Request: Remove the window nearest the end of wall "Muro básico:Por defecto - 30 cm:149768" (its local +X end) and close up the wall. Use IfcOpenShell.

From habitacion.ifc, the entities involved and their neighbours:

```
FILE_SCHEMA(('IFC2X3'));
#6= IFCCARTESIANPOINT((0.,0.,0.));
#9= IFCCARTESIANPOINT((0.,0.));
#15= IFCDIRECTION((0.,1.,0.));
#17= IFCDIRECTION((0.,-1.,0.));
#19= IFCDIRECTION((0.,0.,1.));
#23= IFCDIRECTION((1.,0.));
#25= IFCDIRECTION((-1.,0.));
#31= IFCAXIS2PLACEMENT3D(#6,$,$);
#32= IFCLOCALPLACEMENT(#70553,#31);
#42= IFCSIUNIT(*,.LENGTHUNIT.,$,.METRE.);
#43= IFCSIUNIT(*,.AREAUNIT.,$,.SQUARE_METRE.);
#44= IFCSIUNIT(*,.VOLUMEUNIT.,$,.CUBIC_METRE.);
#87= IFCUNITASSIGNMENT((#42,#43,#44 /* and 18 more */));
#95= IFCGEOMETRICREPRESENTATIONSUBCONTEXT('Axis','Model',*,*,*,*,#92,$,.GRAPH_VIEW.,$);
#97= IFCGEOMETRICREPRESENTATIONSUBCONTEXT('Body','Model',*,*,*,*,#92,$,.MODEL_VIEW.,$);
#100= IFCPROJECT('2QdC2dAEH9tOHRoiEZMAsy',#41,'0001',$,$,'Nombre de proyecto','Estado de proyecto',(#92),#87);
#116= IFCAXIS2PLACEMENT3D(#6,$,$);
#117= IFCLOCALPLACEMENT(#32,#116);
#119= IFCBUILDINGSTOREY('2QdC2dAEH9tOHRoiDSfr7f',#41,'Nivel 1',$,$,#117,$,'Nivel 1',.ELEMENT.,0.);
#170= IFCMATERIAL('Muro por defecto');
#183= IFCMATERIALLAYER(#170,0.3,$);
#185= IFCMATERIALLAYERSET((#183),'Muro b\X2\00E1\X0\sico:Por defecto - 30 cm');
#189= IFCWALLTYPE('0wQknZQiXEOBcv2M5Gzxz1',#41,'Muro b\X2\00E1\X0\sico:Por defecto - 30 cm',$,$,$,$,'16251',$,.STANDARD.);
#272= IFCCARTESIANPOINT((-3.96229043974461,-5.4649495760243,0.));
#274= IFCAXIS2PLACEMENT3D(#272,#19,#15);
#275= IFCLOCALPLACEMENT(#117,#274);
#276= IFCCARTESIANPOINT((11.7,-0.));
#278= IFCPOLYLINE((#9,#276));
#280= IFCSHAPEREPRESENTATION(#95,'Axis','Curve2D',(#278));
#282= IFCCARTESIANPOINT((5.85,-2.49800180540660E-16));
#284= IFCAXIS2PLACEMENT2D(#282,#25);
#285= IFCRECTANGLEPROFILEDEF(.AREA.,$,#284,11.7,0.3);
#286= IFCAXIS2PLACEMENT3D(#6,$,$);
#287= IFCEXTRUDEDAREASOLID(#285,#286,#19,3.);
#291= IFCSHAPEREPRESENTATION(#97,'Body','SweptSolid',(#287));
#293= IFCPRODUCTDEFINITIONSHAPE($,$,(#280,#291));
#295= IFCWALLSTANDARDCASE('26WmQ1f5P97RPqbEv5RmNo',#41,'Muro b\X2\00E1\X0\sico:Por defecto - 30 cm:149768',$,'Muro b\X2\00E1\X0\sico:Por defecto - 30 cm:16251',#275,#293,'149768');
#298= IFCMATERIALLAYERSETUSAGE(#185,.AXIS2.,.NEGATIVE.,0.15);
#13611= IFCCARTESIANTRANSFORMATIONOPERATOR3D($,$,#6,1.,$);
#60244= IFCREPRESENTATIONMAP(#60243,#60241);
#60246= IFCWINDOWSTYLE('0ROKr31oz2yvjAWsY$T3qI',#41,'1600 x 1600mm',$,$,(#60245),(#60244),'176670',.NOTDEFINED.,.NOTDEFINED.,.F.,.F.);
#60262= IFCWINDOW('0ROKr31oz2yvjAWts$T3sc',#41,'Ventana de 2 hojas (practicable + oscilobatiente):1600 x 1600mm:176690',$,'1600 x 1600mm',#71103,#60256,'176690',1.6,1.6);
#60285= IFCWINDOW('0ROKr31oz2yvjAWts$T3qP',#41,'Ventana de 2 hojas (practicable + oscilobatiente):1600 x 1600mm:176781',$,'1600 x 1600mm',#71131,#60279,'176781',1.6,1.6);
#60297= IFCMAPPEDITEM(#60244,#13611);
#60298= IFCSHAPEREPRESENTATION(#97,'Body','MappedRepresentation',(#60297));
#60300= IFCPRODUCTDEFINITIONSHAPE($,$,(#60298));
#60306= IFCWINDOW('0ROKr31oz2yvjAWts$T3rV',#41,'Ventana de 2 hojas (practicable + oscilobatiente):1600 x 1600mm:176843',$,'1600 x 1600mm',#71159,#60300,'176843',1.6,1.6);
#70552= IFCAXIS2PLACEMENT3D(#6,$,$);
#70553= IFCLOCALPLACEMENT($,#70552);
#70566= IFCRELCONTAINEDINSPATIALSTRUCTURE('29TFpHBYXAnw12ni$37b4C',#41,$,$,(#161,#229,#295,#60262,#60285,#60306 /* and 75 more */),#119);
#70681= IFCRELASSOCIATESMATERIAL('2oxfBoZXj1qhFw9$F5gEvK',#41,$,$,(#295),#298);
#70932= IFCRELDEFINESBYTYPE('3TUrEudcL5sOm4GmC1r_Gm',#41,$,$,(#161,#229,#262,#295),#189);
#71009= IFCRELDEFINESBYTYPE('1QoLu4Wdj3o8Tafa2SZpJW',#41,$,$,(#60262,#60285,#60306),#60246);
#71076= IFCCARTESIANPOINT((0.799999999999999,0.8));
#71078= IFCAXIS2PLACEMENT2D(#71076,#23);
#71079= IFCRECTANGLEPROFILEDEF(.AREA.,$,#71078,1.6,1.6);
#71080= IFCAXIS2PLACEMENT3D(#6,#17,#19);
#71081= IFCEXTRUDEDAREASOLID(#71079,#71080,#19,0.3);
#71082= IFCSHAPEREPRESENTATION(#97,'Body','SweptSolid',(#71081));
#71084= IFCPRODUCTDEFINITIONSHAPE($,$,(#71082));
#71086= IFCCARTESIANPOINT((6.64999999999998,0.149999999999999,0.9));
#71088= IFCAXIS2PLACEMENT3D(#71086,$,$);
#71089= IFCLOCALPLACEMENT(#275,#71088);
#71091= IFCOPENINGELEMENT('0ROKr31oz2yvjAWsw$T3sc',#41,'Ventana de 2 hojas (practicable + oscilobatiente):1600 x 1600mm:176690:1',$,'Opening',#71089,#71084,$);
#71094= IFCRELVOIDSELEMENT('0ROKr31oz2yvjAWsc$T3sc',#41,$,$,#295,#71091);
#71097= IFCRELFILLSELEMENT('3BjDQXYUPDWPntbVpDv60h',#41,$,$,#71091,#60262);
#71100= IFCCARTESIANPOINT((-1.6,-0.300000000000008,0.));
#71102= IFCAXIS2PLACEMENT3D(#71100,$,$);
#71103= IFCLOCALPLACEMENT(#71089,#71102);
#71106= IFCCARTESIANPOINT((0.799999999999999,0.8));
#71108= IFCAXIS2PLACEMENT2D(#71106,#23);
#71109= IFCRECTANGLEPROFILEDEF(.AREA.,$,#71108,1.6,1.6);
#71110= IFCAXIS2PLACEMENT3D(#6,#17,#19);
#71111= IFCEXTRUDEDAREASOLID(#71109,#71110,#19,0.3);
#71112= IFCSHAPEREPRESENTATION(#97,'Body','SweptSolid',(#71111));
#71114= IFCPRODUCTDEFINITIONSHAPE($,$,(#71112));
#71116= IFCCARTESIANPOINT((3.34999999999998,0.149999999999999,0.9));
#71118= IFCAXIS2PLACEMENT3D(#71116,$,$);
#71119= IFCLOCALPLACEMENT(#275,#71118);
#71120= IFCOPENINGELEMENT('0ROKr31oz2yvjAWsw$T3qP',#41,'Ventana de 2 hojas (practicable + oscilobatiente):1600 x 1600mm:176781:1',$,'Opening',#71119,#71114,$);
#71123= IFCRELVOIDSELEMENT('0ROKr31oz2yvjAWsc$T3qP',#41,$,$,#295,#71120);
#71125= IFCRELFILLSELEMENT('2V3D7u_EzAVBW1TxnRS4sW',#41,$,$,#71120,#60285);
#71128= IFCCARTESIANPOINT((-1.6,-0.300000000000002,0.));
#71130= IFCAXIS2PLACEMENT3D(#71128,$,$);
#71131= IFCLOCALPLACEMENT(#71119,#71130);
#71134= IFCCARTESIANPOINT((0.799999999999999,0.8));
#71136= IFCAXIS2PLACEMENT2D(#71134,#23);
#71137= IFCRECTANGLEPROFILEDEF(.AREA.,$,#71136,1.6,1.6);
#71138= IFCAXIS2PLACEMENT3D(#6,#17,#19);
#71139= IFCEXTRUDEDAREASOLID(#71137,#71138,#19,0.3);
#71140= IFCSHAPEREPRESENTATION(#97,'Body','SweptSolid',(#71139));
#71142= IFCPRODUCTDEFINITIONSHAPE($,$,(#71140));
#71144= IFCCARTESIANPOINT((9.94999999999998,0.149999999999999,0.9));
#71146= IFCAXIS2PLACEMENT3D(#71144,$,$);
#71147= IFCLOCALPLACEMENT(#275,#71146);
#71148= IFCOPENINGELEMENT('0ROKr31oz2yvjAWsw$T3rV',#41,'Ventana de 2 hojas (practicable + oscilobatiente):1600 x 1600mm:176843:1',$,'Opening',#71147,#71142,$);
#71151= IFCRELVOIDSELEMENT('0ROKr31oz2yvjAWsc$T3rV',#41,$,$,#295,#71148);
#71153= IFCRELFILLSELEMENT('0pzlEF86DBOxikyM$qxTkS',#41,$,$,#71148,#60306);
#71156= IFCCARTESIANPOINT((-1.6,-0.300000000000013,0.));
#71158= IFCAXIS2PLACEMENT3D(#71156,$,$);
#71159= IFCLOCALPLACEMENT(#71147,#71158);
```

```python
import ifcopenshell
import ifcopenshell.api.feature
import ifcopenshell.api.root
import ifcopenshell.geom
import ifcopenshell.util.shape

model = ifcopenshell.open("habitacion.ifc")
settings = ifcopenshell.geom.settings()


def volume(element):
    """Net volume in cubic metres, openings subtracted."""
    shape = ifcopenshell.geom.create_shape(settings, element)
    return ifcopenshell.util.shape.get_volume(shape.geometry)


window = model.by_id(60306)
opening = window.FillsVoids[0].RelatingOpeningElement
wall = opening.VoidsElements[0].RelatingBuildingElement
before = volume(wall)

ifcopenshell.api.root.remove_product(model, product=window)
ifcopenshell.api.feature.remove_feature(model, feature=opening)

after = volume(wall)

print(f"wall volume {before:.3f} -> {after:.3f} m3")

model.write("habitacion_rev.ifc")
```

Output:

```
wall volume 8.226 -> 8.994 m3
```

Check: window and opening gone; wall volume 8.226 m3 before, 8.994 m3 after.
